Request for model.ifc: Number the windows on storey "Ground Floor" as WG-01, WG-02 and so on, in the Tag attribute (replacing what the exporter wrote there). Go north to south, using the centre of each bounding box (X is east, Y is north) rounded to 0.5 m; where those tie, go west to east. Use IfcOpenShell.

First a look at what the model holds.

```python
import ifcopenshell
import ifcopenshell.util.element
import ifcopenshell.util.placement

model = ifcopenshell.open("model.ifc")
print(model.schema)
storey = next(s for s in model.by_type("IfcBuildingStorey") if s.Name == "Ground Floor")
windows = [e for e in ifcopenshell.util.element.get_decomposition(storey) if e.is_a("IfcWindow")]
for e in sorted(windows, key=lambda e: e.id()):
    origin = ifcopenshell.util.placement.get_local_placement(e.ObjectPlacement)[:3, 3]
    print(e.id(), e.Tag, e.Name, origin.round(2) + 0.0, sep=" | ")
```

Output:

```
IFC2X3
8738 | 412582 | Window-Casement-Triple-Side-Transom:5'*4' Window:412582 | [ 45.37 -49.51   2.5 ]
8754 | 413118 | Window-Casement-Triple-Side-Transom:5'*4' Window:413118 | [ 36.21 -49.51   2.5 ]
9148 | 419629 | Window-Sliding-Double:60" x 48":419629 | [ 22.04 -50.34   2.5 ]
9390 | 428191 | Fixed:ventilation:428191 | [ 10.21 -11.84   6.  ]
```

```python
import ifcopenshell
import ifcopenshell.geom
import ifcopenshell.util.element
import ifcopenshell.util.shape

model = ifcopenshell.open("model.ifc")
settings = ifcopenshell.geom.settings()
settings.set("use-world-coords", True)


def centre(element):
    shape = ifcopenshell.geom.create_shape(settings, element)
    return ifcopenshell.util.shape.get_bbox_centroid(shape.geometry)


storey = next(s for s in model.by_type("IfcBuildingStorey") if s.Name == "Ground Floor")
windows = [e for e in ifcopenshell.util.element.get_decomposition(storey) if e.is_a("IfcWindow")]

# Insertion points can sit at a corner or the storey origin, so sort by the geometry (in metres).
centres = {e: centre(e) for e in windows}
windows.sort(key=lambda e: (-round(centres[e][1] / 0.5), centres[e][0]))

for i, e in enumerate(windows, start=1):
    number = f"WG-{i:02d}"
    e.Tag = number
    print(e.id(), number)

model.write("model-out.ifc")
```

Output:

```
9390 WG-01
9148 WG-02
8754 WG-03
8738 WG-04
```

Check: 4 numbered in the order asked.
